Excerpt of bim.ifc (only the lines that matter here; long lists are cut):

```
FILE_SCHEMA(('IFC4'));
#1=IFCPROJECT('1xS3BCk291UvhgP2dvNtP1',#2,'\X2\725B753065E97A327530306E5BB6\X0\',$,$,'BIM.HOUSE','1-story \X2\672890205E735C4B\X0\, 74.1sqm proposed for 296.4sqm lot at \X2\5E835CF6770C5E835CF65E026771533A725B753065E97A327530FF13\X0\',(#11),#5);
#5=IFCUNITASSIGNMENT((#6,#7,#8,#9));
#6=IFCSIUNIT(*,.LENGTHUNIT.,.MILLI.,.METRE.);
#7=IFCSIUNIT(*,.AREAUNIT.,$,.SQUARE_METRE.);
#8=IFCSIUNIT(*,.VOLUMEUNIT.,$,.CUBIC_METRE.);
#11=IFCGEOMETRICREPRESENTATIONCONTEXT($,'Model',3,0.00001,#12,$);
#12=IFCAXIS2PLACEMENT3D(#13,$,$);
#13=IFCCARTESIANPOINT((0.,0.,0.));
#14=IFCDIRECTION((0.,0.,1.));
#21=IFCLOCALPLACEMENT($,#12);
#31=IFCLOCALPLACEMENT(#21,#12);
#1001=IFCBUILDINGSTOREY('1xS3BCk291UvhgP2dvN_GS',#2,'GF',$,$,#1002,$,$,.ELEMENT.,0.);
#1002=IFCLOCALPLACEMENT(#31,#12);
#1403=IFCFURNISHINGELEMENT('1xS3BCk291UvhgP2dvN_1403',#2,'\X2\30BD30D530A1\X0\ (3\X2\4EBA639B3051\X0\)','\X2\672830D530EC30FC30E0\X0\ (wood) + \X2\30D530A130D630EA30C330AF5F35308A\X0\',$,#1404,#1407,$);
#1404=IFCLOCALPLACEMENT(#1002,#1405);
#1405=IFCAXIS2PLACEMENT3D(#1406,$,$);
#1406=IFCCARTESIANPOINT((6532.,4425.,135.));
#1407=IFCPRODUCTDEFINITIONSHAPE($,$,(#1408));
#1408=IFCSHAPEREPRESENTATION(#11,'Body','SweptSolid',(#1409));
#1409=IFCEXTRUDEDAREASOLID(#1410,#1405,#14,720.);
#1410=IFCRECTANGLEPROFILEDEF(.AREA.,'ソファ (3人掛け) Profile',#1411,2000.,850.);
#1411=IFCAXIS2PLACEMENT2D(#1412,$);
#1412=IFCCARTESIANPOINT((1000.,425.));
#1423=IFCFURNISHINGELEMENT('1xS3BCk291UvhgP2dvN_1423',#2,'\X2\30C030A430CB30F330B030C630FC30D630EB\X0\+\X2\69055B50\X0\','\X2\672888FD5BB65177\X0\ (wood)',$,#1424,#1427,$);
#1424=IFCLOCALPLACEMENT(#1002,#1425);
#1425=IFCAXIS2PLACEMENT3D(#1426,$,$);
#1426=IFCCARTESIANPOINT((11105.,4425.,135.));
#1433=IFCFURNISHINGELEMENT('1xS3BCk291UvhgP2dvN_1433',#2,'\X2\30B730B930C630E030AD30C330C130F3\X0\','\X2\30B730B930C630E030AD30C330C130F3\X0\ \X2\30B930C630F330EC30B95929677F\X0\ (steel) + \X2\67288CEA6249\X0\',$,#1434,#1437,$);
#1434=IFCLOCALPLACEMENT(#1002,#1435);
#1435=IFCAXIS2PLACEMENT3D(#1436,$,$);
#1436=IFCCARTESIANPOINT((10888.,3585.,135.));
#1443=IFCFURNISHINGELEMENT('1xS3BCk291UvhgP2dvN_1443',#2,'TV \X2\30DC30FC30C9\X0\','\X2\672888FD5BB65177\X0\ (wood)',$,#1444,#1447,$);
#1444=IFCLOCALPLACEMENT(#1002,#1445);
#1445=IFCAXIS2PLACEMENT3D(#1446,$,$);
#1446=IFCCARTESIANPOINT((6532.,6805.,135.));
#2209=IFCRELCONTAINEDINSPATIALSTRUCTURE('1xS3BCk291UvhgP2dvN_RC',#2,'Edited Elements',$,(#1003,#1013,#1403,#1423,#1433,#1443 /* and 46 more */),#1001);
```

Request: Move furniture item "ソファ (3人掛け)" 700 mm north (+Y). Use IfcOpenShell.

```python
import ifcopenshell
import ifcopenshell.api.geometry
import ifcopenshell.util.placement
import ifcopenshell.util.unit

model = ifcopenshell.open("bim.ifc")
unit_scale = ifcopenshell.util.unit.calculate_unit_scale(model)

item = model.by_guid("1xS3BCk291UvhgP2dvN_1403")
matrix = ifcopenshell.util.placement.get_local_placement(item.ObjectPlacement)
matrix[1, 3] += 0.7 / unit_scale
ifcopenshell.api.geometry.edit_object_placement(model, product=item, matrix=matrix, is_si=False)

print(ifcopenshell.util.placement.get_local_placement(item.ObjectPlacement).round(3) + 0.0)

model.write("bim-out.ifc")
```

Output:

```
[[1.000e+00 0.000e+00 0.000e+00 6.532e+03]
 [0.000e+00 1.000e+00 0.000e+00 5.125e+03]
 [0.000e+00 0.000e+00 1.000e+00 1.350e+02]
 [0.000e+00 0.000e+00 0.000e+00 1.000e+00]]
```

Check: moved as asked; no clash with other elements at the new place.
